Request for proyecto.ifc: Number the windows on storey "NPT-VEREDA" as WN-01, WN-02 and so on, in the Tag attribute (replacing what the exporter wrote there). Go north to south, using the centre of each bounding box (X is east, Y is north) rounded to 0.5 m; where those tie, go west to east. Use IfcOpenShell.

First a look at what the model holds.

```python
import ifcopenshell
import ifcopenshell.util.element
import ifcopenshell.util.placement

model = ifcopenshell.open("proyecto.ifc")
print(model.schema)
storey = next(s for s in model.by_type("IfcBuildingStorey") if s.Name == "NPT-VEREDA")
windows = [e for e in ifcopenshell.util.element.get_decomposition(storey) if e.is_a("IfcWindow")]
for e in sorted(windows, key=lambda e: e.id()):
    origin = ifcopenshell.util.placement.get_local_placement(e.ObjectPlacement)[:3, 3]
    print(e.id(), e.Tag, e.Name, origin.round(2) + 0.0, sep=" | ")
```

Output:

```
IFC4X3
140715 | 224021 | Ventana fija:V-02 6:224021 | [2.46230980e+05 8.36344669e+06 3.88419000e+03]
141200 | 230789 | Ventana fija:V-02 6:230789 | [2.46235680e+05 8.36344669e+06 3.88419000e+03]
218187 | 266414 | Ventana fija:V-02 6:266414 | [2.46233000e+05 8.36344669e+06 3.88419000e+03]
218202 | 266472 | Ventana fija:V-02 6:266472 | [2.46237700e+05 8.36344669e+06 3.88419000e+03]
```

```python
import ifcopenshell
import ifcopenshell.geom
import ifcopenshell.util.element
import ifcopenshell.util.shape

model = ifcopenshell.open("proyecto.ifc")
settings = ifcopenshell.geom.settings()
settings.set("use-world-coords", True)


def centre(element):
    shape = ifcopenshell.geom.create_shape(settings, element)
    return ifcopenshell.util.shape.get_bbox_centroid(shape.geometry)


storey = next(s for s in model.by_type("IfcBuildingStorey") if s.Name == "NPT-VEREDA")
windows = [e for e in ifcopenshell.util.element.get_decomposition(storey) if e.is_a("IfcWindow")]

# Insertion points can sit at a corner or the storey origin, so sort by the geometry (in metres).
centres = {e: centre(e) for e in windows}
windows.sort(key=lambda e: (-round(centres[e][1] / 0.5), centres[e][0]))

for i, e in enumerate(windows, start=1):
    number = f"WN-{i:02d}"
    e.Tag = number
    print(e.id(), number)

model.write("proyecto-out.ifc")
```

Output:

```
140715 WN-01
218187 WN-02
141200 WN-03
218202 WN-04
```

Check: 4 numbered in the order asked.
